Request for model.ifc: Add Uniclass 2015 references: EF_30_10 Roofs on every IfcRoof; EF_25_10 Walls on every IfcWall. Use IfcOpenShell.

First a look at what the model holds.

```python
import ifcopenshell

model = ifcopenshell.open("model.ifc")
print(model.schema)
print("classifications:", [c.Name for c in model.by_type("IfcClassification")])
for ifc_class in ("IfcDoor", "IfcRoof", "IfcStair", "IfcWall", "IfcWindow"):
    print(ifc_class, len(model.by_type(ifc_class)))
```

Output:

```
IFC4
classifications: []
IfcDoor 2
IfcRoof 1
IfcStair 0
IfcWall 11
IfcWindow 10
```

```python
import ifcopenshell
import ifcopenshell.api.classification

model = ifcopenshell.open("model.ifc")

system = ifcopenshell.api.classification.add_classification(model, classification="Uniclass 2015")

codes = {
    "IfcRoof": ("EF_30_10", "Roofs"),
    "IfcWall": ("EF_25_10", "Walls"),
}
for ifc_class, (code, name) in codes.items():
    products = model.by_type(ifc_class)
    ifcopenshell.api.classification.add_reference(
        model, products=products, classification=system, identification=code, name=name
    )
    print(code, len(products))

model.write("model-out.ifc")
```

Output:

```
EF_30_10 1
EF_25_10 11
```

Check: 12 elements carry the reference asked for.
